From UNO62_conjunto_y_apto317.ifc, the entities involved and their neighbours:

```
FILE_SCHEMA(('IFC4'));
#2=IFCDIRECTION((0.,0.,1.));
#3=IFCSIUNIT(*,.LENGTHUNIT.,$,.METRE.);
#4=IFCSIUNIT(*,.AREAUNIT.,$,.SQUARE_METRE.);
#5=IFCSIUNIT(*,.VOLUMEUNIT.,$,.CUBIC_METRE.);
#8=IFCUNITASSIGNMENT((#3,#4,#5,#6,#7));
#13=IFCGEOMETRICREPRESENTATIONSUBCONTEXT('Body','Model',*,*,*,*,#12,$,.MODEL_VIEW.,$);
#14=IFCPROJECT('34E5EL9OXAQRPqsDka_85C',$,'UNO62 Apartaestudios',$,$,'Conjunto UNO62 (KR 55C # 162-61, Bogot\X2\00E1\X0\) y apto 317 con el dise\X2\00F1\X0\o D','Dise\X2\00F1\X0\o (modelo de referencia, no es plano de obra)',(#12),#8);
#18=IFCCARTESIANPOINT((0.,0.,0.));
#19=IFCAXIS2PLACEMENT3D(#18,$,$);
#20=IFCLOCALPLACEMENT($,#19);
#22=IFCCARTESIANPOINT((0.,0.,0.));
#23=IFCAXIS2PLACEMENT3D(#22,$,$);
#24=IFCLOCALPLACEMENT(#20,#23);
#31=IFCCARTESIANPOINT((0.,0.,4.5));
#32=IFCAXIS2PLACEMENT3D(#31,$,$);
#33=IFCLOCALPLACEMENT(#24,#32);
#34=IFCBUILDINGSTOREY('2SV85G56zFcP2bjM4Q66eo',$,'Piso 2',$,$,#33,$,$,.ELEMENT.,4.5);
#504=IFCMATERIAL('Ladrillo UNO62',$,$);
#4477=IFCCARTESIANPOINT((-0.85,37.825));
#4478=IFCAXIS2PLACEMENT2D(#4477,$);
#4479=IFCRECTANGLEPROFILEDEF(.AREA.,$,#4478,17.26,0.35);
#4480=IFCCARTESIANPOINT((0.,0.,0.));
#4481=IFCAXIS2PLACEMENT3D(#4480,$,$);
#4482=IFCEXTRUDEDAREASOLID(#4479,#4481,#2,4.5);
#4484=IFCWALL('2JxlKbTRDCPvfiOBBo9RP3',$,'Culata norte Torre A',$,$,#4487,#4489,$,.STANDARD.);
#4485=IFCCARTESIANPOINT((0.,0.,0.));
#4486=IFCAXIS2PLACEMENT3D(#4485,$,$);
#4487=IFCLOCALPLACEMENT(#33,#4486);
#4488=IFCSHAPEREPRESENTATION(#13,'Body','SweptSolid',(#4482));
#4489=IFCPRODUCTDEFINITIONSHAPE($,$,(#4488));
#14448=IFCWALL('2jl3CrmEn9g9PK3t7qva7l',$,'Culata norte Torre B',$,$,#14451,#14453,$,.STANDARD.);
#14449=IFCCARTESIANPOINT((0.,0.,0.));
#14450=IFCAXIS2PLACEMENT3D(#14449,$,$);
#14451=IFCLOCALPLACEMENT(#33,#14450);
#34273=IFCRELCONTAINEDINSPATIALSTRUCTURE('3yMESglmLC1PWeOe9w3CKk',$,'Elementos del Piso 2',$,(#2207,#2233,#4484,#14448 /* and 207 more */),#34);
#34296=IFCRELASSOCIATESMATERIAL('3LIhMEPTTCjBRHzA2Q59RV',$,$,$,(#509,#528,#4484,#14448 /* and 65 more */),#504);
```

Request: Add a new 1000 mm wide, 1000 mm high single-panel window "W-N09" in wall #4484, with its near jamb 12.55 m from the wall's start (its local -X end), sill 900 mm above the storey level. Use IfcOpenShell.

```python
import numpy as np
import ifcopenshell
import ifcopenshell.api.feature
import ifcopenshell.api.geometry
import ifcopenshell.api.root
import ifcopenshell.api.spatial
import ifcopenshell.geom
import ifcopenshell.util.element
import ifcopenshell.util.placement
import ifcopenshell.util.representation
import ifcopenshell.util.shape
import ifcopenshell.util.unit

model = ifcopenshell.open("UNO62_conjunto_y_apto317.ifc")
unit_scale = ifcopenshell.util.unit.calculate_unit_scale(model)
settings = ifcopenshell.geom.settings()


def volume(element):
    """Net volume in cubic metres, openings subtracted."""
    shape = ifcopenshell.geom.create_shape(settings, element)
    return ifcopenshell.util.shape.get_volume(shape.geometry)


wall = model.by_guid("2JxlKbTRDCPvfiOBBo9RP3")
storey = ifcopenshell.util.element.get_container(wall, ifc_class="IfcBuildingStorey")
context = ifcopenshell.util.representation.get_context(model, "Model", "Body", "MODEL_VIEW")
before = volume(wall)

width, height, from_end, sill = 1, 1, 12.55, 0.9  # metres

# The wall runs along its own X axis, and the end named is its -X end.
wall_shape = ifcopenshell.geom.create_shape(settings, wall)
x, y, z = ifcopenshell.util.shape.get_vertices(wall_shape.geometry).T
start = x.min() + from_end
face, thickness = float(y.min()), float(y.max() - y.min())
wall_matrix = ifcopenshell.util.placement.get_local_placement(wall.ObjectPlacement)
level = ifcopenshell.util.placement.get_local_placement(storey.ObjectPlacement)[2, 3]


def in_wall(x, y):
    """Placement at x, y metres in the wall's axes, at sill height."""
    matrix = wall_matrix.copy()
    matrix[:, 3] = wall_matrix @ np.array([x / unit_scale, y / unit_scale, 0.0, 1.0])
    matrix[2, 3] = level + sill / unit_scale
    return matrix


# Opening: a box that overshoots both wall faces by 50 mm.
opening = ifcopenshell.api.root.create_entity(model, ifc_class="IfcOpeningElement", predefined_type="OPENING")
box = ifcopenshell.api.geometry.add_wall_representation(
    model, context=context, length=width, height=height, thickness=thickness + 0.1
)
ifcopenshell.api.geometry.assign_representation(model, product=opening, representation=box)
ifcopenshell.api.geometry.edit_object_placement(model, product=opening, matrix=in_wall(start, face - 0.05), is_si=False)
ifcopenshell.api.feature.add_feature(model, feature=opening, element=wall)

window = ifcopenshell.api.root.create_entity(model, ifc_class="IfcWindow", name="W-N09", predefined_type="WINDOW")
window.OverallWidth, window.OverallHeight = width / unit_scale, height / unit_scale
window.PartitioningType = "SINGLE_PANEL"
body = ifcopenshell.api.geometry.add_window_representation(
    model,
    context=context,
    overall_width=window.OverallWidth,
    overall_height=window.OverallHeight,
    partition_type="SINGLE_PANEL",
)
ifcopenshell.api.geometry.assign_representation(model, product=window, representation=body)
ifcopenshell.api.spatial.assign_container(model, products=[window], relating_structure=storey)
ifcopenshell.api.feature.add_filling(model, opening=opening, element=window)

# Centre the window in the wall's thickness.
ifcopenshell.api.geometry.edit_object_placement(model, product=window, matrix=in_wall(start, face), is_si=False)
window_shape = ifcopenshell.geom.create_shape(settings, window)
depth = ifcopenshell.util.shape.get_vertices(window_shape.geometry)[:, 1]
offset = face + thickness / 2 - (depth.min() + depth.max()) / 2
ifcopenshell.api.geometry.edit_object_placement(model, product=window, matrix=in_wall(start, offset), is_si=False)

after = volume(wall)

print(f"wall volume {before:.3f} -> {after:.3f} m3")

model.write("UNO62_conjunto_y_apto317-out.ifc")
```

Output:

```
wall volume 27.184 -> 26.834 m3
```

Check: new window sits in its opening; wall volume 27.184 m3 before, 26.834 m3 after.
